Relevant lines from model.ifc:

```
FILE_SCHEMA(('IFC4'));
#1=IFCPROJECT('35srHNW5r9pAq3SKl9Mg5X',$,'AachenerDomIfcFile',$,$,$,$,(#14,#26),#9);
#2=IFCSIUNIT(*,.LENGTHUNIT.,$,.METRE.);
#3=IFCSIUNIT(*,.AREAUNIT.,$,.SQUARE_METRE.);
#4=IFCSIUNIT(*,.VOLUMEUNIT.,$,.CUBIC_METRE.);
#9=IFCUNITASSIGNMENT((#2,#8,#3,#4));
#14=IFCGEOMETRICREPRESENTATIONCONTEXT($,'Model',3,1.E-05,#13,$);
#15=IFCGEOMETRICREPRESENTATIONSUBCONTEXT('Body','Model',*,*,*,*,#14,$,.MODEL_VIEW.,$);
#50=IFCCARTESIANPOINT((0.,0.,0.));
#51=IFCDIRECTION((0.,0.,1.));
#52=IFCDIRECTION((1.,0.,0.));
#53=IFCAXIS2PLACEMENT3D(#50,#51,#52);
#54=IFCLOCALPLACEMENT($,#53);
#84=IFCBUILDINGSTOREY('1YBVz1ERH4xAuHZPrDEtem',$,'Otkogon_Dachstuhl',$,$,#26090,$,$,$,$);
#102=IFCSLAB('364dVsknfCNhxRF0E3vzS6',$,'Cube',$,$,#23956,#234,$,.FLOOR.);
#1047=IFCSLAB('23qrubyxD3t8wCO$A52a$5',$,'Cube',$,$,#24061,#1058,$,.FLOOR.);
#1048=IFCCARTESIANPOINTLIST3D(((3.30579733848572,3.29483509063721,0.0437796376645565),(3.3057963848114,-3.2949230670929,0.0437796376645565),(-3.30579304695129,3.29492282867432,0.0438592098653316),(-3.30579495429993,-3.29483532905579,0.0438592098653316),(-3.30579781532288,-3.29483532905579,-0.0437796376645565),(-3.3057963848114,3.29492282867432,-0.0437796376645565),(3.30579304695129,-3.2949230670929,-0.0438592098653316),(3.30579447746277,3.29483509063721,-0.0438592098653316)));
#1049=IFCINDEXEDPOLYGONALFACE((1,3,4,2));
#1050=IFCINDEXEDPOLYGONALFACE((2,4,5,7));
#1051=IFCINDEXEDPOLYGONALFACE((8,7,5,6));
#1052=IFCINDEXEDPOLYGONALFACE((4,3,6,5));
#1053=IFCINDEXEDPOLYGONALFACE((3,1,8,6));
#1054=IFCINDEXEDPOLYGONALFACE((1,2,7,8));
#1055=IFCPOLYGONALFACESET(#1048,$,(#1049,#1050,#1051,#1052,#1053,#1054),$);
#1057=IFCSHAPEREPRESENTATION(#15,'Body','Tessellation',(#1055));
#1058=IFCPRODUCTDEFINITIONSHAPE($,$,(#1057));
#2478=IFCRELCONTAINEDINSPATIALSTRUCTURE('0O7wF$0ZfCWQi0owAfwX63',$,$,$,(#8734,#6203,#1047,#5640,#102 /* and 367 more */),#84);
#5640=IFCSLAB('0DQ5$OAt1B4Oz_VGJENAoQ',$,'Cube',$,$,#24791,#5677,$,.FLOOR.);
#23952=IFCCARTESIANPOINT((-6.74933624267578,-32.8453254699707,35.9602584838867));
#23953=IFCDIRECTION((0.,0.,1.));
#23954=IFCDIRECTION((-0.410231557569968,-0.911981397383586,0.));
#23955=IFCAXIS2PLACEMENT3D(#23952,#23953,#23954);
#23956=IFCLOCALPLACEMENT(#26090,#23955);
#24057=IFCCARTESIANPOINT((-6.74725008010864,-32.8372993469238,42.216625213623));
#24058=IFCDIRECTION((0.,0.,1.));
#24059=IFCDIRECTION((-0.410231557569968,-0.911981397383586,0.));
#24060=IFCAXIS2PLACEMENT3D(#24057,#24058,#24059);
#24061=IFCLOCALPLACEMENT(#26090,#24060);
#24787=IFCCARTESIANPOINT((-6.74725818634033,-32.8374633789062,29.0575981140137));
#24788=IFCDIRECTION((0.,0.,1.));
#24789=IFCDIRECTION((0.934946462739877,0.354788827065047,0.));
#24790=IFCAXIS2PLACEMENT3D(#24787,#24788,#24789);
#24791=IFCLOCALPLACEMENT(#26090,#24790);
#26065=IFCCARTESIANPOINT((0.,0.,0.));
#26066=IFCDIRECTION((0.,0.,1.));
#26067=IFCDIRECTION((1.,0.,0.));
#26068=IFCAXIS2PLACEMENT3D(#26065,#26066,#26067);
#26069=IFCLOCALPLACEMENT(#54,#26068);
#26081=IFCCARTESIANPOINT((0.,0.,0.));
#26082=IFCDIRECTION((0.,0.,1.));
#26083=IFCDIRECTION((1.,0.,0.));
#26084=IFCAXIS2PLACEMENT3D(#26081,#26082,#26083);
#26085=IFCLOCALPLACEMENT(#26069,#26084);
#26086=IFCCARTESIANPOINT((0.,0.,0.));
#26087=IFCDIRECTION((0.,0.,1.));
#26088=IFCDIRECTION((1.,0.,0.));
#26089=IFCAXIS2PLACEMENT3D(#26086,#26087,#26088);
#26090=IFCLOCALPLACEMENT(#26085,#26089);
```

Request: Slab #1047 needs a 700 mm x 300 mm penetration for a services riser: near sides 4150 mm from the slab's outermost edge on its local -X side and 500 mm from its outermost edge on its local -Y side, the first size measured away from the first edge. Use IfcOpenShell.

```python
import numpy as np
import ifcopenshell
import ifcopenshell.api.feature
import ifcopenshell.api.geometry
import ifcopenshell.api.root
import ifcopenshell.geom
import ifcopenshell.util.placement
import ifcopenshell.util.representation
import ifcopenshell.util.shape
import ifcopenshell.util.unit

model = ifcopenshell.open("model.ifc")
unit_scale = ifcopenshell.util.unit.calculate_unit_scale(model)
settings = ifcopenshell.geom.settings()


def volume(element):
    """Net volume in cubic metres, openings subtracted."""
    shape = ifcopenshell.geom.create_shape(settings, element)
    return ifcopenshell.util.shape.get_volume(shape.geometry)


slab = model.by_guid("23qrubyxD3t8wCO$A52a$5")
before = volume(slab)

# Extent in the slab's own axes, in metres. The edges named are its -X and -Y sides.
slab_shape = ifcopenshell.geom.create_shape(settings, slab)
vertices = ifcopenshell.util.shape.get_vertices(slab_shape.geometry)
x_min, y_min, bottom = vertices.min(axis=0)
top = vertices[:, 2].max()

opening = ifcopenshell.api.root.create_entity(model, ifc_class="IfcOpeningElement", name="Services riser opening", predefined_type="OPENING")
context = ifcopenshell.util.representation.get_context(model, "Model", "Body", "MODEL_VIEW")
width, depth = 0.7, 0.3
outline = [(0.0, 0.0), (width, 0.0), (width, depth), (0.0, depth), (0.0, 0.0)]
# Overshoot both faces by 50 mm so the cut is clean.
shape = ifcopenshell.api.geometry.add_slab_representation(
    model, context=context, depth=top - bottom + 0.1, polyline=outline
)
ifcopenshell.api.geometry.assign_representation(model, product=opening, representation=shape)

matrix = ifcopenshell.util.placement.get_local_placement(slab.ObjectPlacement)
matrix[:, 3] = matrix @ np.append(np.array([x_min + 4.15, y_min + 0.5, bottom - 0.05]) / unit_scale, 1.0)
ifcopenshell.api.geometry.edit_object_placement(model, product=opening, matrix=matrix, is_si=False)
ifcopenshell.api.feature.add_feature(model, feature=opening, element=slab)

after = volume(slab)

print(f"slab volume {before:.3f} -> {after:.3f} m3")

model.write("model_v2.ifc")
```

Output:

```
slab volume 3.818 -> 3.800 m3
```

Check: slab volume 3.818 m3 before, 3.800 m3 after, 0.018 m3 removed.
